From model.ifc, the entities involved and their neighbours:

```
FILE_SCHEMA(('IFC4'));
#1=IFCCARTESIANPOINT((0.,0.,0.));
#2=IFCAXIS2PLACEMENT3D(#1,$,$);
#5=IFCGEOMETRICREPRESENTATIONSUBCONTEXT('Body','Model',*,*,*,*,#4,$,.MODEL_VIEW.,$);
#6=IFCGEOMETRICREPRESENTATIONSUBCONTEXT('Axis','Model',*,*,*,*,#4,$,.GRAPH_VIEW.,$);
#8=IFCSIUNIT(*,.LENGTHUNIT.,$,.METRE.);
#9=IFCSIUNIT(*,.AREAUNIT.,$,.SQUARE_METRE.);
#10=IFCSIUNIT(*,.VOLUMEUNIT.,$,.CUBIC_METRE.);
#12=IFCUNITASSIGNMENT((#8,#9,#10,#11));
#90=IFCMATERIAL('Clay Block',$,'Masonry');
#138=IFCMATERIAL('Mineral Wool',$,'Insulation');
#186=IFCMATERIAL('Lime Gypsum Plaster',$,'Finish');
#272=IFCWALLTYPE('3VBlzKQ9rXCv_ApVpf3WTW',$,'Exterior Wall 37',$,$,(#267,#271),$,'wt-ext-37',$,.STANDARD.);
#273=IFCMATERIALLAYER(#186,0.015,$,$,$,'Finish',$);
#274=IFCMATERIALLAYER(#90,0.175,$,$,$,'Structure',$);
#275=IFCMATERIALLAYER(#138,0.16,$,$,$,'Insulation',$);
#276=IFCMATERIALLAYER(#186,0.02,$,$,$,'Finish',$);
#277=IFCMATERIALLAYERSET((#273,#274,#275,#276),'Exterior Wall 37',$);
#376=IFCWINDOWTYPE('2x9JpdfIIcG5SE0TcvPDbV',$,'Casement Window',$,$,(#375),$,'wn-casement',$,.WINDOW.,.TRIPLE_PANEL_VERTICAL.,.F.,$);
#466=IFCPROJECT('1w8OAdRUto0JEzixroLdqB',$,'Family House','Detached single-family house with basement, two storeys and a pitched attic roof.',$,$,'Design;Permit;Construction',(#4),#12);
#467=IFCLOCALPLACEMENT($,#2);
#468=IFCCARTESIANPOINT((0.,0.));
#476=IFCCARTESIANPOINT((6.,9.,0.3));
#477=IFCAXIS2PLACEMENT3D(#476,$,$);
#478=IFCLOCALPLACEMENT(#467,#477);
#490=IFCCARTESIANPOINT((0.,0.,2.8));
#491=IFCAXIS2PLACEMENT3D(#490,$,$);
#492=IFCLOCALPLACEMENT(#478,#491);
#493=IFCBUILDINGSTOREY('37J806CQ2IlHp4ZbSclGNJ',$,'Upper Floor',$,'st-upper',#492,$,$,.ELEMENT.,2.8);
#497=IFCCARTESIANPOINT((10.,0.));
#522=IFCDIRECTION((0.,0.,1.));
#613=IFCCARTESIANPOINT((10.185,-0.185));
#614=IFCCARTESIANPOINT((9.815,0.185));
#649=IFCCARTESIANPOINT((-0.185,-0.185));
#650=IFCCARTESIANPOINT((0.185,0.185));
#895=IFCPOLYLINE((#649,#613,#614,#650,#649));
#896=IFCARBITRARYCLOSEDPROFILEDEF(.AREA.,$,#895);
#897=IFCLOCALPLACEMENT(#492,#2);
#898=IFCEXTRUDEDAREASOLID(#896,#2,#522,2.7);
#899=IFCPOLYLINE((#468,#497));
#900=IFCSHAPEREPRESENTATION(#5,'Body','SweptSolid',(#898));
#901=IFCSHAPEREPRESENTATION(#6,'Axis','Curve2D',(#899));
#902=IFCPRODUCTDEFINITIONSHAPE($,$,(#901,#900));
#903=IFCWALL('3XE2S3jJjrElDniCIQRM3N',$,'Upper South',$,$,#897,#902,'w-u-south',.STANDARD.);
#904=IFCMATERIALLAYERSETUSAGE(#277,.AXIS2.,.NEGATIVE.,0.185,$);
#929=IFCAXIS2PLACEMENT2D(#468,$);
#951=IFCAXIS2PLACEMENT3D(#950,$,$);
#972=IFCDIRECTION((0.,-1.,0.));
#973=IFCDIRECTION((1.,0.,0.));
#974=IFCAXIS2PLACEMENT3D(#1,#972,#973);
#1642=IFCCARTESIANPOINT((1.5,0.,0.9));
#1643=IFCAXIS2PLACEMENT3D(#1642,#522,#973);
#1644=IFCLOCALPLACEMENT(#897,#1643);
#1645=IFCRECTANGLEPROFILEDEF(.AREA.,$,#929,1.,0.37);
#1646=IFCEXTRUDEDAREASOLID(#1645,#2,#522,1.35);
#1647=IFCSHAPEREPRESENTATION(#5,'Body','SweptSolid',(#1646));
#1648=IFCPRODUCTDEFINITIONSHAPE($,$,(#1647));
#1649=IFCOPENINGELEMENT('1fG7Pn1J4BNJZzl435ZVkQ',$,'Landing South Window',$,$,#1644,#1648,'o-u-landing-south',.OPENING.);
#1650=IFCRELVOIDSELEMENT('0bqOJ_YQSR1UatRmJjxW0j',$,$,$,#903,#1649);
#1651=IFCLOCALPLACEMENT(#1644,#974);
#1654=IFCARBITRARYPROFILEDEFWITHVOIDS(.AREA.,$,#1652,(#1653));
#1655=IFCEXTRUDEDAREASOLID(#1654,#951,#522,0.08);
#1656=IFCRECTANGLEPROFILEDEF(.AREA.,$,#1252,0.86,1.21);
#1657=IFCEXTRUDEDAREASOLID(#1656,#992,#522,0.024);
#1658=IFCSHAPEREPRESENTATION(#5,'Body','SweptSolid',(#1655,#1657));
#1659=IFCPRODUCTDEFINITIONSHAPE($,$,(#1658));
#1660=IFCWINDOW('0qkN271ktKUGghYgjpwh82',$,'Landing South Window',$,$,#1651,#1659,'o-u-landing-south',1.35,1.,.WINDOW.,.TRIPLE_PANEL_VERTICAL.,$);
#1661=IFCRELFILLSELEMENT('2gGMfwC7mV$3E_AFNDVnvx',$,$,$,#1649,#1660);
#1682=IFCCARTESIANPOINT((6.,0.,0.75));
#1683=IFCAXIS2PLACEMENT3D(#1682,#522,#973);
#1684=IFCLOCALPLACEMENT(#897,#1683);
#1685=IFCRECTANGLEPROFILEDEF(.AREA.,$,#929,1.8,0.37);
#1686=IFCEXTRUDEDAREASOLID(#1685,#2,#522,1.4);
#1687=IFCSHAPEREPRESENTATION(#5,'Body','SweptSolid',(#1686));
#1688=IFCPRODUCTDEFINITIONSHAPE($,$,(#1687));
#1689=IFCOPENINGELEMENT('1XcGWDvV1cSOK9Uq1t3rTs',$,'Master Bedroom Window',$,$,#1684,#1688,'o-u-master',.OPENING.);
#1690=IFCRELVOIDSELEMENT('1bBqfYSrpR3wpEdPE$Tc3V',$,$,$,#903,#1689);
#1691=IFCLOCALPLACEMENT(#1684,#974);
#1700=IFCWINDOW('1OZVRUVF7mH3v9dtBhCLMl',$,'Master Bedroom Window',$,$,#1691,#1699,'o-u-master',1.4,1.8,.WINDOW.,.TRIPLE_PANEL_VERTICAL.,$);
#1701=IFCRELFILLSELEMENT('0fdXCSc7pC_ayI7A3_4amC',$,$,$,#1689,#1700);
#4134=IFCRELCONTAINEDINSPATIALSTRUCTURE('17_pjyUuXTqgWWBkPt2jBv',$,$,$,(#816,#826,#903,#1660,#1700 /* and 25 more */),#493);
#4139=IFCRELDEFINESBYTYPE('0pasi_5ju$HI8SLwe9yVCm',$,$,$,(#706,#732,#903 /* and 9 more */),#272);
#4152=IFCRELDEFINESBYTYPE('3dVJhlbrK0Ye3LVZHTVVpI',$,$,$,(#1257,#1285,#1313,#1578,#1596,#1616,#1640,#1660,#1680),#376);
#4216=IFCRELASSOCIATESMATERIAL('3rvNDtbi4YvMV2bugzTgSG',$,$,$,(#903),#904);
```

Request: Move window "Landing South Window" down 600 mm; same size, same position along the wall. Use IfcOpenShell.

```python
import numpy as np
import ifcopenshell
import ifcopenshell.api.geometry
import ifcopenshell.util.placement
import ifcopenshell.util.unit

model = ifcopenshell.open("model.ifc")
unit_scale = ifcopenshell.util.unit.calculate_unit_scale(model)

window = model.by_id(1660)
opening = window.FillsVoids[0].RelatingOpeningElement
dz = -0.6 / unit_scale

shift = np.array([0.0, 0.0, dz])
# The window is placed relative to its opening, so it follows when the opening moves.
matrix = ifcopenshell.util.placement.get_local_placement(opening.ObjectPlacement)
matrix[:3, 3] += shift
ifcopenshell.api.geometry.edit_object_placement(
    model, product=opening, matrix=matrix, is_si=False, should_transform_children=True
)

print(f"moved by {dz * unit_scale:+.3f} m")

model.write("model_edited.ifc")
```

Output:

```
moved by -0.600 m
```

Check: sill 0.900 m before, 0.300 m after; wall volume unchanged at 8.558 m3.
